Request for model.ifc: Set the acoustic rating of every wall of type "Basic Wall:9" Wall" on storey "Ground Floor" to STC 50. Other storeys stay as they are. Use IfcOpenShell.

First a look at what the model holds.

```python
import ifcopenshell
import ifcopenshell.util.element

model = ifcopenshell.open("model.ifc")
print(model.schema)
storey = next(s for s in model.by_type("IfcBuildingStorey") if s.Name == "Ground Floor")
walls = [e for e in ifcopenshell.util.element.get_decomposition(storey) if e.is_a("IfcWall")]
seen = {}
for e in walls:
    element_type = ifcopenshell.util.element.get_type(e)
    key = (element_type.Name if element_type != e and element_type else None, ifcopenshell.util.element.get_pset(e, "Pset_WallCommon", "AcousticRating"))
    seen[key] = seen.get(key, 0) + 1
for (name, value), count in sorted(seen.items(), key=str):
    print(count, "x", name, "|", value)
```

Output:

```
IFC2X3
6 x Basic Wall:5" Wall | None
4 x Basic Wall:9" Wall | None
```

```python
import ifcopenshell
import ifcopenshell.api.pset
import ifcopenshell.util.element

model = ifcopenshell.open("model.ifc")

storey = next(s for s in model.by_type("IfcBuildingStorey") if s.Name == "Ground Floor")
walls = [e for e in ifcopenshell.util.element.get_decomposition(storey) if e.is_a("IfcWall")]

count = 0
for e in walls:
    element_type = ifcopenshell.util.element.get_type(e)
    if element_type in (None, e) or element_type.Name != 'Basic Wall:9" Wall':
        continue
    # add_pset returns the element's existing set when there is one.
    pset = ifcopenshell.api.pset.add_pset(model, product=e, name="Pset_WallCommon")
    ifcopenshell.api.pset.edit_pset(model, pset=pset, properties={"AcousticRating": "STC 50"})
    count += 1

print(count, "walls updated")

model.write("model_edited.ifc")
```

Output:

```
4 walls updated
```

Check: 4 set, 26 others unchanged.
